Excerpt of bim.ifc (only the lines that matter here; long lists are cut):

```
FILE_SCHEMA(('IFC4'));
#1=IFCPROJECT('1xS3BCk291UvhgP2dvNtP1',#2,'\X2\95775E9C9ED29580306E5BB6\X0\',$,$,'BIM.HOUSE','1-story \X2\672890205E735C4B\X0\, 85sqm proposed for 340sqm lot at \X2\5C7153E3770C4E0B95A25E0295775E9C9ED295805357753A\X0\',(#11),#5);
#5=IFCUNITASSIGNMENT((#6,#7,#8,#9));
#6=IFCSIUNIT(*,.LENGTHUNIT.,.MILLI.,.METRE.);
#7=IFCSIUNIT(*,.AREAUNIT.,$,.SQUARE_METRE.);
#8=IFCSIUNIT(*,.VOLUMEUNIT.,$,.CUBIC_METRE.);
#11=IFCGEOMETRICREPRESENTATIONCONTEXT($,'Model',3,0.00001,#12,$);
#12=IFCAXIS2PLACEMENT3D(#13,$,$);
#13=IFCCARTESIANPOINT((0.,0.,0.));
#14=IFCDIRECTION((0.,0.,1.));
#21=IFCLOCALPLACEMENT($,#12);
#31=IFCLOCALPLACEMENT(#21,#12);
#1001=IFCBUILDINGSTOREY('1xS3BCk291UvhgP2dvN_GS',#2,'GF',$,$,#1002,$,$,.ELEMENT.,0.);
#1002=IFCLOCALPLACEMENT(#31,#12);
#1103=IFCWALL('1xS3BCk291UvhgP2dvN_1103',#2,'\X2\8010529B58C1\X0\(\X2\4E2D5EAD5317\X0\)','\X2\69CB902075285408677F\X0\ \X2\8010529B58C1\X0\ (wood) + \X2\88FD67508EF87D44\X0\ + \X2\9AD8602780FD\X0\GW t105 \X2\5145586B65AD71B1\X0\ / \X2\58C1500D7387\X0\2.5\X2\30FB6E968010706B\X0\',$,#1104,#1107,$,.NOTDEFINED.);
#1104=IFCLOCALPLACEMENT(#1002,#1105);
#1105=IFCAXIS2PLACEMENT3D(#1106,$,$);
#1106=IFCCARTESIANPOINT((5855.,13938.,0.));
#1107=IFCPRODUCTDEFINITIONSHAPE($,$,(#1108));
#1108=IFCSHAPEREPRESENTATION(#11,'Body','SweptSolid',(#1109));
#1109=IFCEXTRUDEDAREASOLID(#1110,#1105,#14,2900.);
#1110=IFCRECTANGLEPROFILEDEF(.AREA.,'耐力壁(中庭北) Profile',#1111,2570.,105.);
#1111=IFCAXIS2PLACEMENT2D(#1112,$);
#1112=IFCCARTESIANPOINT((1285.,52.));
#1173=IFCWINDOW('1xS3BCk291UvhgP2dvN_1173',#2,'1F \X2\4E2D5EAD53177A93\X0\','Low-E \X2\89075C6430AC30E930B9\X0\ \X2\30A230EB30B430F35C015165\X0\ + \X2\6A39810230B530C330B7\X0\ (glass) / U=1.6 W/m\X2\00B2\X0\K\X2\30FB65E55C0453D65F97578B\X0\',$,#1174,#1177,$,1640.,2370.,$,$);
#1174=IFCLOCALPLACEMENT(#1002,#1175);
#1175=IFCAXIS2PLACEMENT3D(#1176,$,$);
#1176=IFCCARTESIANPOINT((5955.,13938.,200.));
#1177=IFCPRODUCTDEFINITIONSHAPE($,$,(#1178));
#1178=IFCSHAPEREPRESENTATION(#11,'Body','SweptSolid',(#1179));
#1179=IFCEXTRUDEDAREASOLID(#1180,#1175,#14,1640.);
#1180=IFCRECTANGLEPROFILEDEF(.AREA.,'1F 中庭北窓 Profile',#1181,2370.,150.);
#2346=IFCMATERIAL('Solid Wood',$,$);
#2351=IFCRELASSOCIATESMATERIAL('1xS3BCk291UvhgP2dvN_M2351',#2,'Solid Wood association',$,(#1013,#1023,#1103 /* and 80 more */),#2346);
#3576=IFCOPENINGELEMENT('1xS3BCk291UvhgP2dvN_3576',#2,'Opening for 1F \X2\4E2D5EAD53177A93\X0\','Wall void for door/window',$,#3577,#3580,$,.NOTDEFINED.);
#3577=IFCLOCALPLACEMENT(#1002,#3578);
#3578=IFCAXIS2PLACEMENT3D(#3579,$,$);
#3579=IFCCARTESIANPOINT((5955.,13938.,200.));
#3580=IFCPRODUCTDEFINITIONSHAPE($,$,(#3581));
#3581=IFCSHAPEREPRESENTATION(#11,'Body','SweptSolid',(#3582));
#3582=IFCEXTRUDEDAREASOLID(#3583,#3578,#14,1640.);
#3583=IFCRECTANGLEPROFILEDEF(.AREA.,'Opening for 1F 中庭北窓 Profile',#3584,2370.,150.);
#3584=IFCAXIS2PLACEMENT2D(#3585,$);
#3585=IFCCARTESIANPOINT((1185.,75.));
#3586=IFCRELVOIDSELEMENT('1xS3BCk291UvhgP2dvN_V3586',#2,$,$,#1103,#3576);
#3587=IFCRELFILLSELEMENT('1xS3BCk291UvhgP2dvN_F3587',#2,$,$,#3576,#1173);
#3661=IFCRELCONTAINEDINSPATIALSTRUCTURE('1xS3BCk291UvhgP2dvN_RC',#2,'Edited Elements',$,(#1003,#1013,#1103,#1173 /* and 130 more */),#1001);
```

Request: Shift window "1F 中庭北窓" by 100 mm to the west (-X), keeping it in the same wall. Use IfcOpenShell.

```python
import ifcopenshell
import ifcopenshell.api.geometry
import ifcopenshell.util.placement

model = ifcopenshell.open("bim.ifc")

window = model.by_guid("1xS3BCk291UvhgP2dvN_1173")
opening = window.FillsVoids[0].RelatingOpeningElement
wall = opening.VoidsElements[0].RelatingBuildingElement

wall_matrix = ifcopenshell.util.placement.get_local_placement(wall.ObjectPlacement)
shift = wall_matrix[:3, 0] * -100.0
before = ifcopenshell.util.placement.get_local_placement(window.ObjectPlacement)[:3, 3].copy()

# The window is not placed relative to its opening, so move both.
for product in (opening, window):
    matrix = ifcopenshell.util.placement.get_local_placement(product.ObjectPlacement)
    matrix[:3, 3] += shift
    ifcopenshell.api.geometry.edit_object_placement(model, product=product, matrix=matrix, is_si=False)

after = ifcopenshell.util.placement.get_local_placement(window.ObjectPlacement)[:3, 3]
print("window moved by", (after - before).round(3) + 0.0)

model.write("bim_rev.ifc")
```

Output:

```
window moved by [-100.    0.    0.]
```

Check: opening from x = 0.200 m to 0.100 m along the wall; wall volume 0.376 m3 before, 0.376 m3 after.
